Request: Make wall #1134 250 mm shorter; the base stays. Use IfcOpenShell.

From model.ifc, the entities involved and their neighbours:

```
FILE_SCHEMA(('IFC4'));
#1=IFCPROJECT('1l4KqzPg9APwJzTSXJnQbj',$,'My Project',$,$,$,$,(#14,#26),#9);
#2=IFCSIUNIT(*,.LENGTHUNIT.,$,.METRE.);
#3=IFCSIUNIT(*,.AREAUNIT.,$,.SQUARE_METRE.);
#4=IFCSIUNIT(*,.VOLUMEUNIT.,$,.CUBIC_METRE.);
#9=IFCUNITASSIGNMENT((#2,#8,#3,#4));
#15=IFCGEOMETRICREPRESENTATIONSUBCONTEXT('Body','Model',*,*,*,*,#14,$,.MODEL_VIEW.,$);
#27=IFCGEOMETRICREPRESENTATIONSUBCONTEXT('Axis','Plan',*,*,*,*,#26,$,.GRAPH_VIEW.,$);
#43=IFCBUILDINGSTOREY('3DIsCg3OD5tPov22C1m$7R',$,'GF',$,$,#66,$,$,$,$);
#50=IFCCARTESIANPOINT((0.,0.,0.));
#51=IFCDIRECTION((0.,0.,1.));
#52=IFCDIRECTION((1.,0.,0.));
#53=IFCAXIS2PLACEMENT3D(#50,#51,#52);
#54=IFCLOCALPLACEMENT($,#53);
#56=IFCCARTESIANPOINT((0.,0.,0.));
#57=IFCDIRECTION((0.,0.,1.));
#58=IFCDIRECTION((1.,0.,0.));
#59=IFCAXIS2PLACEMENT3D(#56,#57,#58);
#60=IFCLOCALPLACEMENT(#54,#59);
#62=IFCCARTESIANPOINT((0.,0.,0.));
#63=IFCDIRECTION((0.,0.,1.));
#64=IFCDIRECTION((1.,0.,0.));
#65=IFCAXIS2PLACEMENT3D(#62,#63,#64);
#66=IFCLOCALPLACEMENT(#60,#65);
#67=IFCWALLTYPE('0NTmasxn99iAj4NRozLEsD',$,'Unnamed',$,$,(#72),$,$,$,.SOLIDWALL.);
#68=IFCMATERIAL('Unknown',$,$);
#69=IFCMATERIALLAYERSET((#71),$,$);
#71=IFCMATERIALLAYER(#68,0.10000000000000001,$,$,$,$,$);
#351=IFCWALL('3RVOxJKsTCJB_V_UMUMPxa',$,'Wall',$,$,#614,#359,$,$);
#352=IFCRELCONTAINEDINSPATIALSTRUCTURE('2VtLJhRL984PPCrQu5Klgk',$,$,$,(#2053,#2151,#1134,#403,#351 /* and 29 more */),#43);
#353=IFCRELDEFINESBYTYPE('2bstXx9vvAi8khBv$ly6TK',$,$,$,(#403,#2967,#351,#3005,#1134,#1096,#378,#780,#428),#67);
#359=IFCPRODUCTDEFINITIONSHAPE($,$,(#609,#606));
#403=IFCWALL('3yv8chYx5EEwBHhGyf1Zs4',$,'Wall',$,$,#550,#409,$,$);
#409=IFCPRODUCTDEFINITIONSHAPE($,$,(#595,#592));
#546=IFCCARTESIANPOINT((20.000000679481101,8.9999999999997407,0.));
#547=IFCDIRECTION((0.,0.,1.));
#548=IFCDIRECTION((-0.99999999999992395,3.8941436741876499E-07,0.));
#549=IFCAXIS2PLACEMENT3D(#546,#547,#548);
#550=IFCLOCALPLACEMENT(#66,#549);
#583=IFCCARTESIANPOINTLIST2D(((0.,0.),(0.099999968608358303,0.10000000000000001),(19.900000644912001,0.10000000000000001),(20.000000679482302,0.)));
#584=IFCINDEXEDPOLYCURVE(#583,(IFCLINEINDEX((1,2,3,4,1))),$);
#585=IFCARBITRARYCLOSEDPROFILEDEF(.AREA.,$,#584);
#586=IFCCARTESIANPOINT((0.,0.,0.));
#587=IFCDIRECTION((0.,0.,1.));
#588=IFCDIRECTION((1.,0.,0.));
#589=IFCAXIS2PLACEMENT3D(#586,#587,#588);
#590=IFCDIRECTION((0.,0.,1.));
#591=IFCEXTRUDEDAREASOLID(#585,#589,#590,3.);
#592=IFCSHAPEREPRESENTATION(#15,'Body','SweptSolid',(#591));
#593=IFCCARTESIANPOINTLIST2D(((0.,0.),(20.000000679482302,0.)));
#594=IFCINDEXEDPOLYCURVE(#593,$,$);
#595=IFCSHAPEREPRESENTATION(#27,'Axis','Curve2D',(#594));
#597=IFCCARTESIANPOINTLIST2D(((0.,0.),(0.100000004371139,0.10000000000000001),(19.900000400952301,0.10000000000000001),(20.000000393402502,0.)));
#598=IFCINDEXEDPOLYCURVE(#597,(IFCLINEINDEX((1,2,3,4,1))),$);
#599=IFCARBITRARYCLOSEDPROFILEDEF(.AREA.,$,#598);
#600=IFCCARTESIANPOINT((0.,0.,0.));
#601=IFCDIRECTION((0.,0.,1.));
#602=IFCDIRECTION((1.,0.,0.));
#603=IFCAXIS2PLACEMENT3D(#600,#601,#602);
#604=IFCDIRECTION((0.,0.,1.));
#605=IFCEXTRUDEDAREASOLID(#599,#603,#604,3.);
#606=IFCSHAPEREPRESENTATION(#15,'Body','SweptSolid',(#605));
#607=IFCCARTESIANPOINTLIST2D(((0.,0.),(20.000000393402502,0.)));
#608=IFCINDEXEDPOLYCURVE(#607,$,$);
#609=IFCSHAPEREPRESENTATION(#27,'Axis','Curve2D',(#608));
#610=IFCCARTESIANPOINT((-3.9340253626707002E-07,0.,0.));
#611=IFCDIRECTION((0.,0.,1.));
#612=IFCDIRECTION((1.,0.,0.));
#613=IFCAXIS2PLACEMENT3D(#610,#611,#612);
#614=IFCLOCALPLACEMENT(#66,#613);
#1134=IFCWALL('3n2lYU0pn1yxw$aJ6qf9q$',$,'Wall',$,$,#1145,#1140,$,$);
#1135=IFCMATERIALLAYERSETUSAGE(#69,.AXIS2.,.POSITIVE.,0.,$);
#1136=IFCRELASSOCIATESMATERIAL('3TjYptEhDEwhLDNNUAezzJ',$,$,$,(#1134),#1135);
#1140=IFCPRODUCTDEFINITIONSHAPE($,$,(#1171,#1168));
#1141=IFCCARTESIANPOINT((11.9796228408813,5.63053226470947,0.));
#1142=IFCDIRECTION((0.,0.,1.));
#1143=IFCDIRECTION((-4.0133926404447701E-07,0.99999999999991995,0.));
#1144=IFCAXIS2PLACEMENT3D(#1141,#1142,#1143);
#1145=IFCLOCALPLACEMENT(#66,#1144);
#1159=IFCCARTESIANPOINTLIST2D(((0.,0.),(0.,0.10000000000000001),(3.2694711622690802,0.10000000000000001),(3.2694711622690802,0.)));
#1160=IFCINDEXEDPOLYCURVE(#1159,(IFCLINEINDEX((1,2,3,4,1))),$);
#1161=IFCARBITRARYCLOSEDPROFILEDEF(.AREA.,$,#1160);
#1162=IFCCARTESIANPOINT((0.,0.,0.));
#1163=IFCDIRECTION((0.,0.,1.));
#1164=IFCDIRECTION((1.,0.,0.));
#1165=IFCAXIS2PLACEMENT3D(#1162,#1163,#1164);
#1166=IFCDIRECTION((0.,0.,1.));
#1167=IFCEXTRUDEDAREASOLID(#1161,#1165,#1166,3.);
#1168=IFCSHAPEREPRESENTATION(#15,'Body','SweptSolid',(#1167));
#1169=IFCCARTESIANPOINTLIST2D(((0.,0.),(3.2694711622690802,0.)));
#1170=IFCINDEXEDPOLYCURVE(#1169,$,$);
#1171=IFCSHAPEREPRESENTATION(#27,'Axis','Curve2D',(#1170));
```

```python
import ifcopenshell
import ifcopenshell.geom
import ifcopenshell.util.representation
import ifcopenshell.util.shape

model = ifcopenshell.open("model.ifc")
settings = ifcopenshell.geom.settings()


def volume(element):
    """Net volume in cubic metres, openings subtracted."""
    shape = ifcopenshell.geom.create_shape(settings, element)
    return ifcopenshell.util.shape.get_volume(shape.geometry)


wall = model.by_id(1134)
before = volume(wall)

body = ifcopenshell.util.representation.get_representation(wall, "Model", "Body")
solid = body.Items[0]
old_height = solid.Depth
solid.Depth -= 0.25
after = volume(wall)

print(f"height {old_height:g} -> {solid.Depth:g}, volume {before:.3f} -> {after:.3f} m3")

model.write("model_edited.ifc")
```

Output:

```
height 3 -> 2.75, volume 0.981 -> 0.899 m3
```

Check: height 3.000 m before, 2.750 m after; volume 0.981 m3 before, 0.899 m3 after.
